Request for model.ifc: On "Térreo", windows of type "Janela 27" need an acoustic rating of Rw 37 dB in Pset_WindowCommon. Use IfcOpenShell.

First a look at what the model holds.

```python
import ifcopenshell
import ifcopenshell.util.element

model = ifcopenshell.open("model.ifc")
print(model.schema)
storey = next(s for s in model.by_type("IfcBuildingStorey") if s.Name == "Térreo")
windows = [e for e in ifcopenshell.util.element.get_decomposition(storey) if e.is_a("IfcWindow")]
seen = {}
for e in windows:
    element_type = ifcopenshell.util.element.get_type(e)
    key = (element_type.Name if element_type != e and element_type else None, ifcopenshell.util.element.get_pset(e, "Pset_WindowCommon", "AcousticRating"))
    seen[key] = seen.get(key, 0) + 1
for (name, value), count in sorted(seen.items(), key=str):
    print(count, "x", name, "|", value)
```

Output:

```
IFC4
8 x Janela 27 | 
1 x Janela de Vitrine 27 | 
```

```python
import ifcopenshell
import ifcopenshell.api.pset
import ifcopenshell.util.element

model = ifcopenshell.open("model.ifc")

storey = next(s for s in model.by_type("IfcBuildingStorey") if s.Name == "Térreo")
windows = [e for e in ifcopenshell.util.element.get_decomposition(storey) if e.is_a("IfcWindow")]

count = 0
for e in windows:
    element_type = ifcopenshell.util.element.get_type(e)
    if element_type in (None, e) or element_type.Name != "Janela 27":
        continue
    # add_pset returns the element's existing set when there is one.
    pset = ifcopenshell.api.pset.add_pset(model, product=e, name="Pset_WindowCommon")
    ifcopenshell.api.pset.edit_pset(model, pset=pset, properties={"AcousticRating": "Rw 37 dB"})
    count += 1

print(count, "windows updated")

model.write("model_updated.ifc")
```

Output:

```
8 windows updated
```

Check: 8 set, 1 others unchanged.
